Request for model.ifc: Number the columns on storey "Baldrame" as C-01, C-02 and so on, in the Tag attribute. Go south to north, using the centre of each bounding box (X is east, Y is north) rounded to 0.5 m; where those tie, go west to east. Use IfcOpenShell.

First a look at what the model holds.

```python
import ifcopenshell
import ifcopenshell.util.element
import ifcopenshell.util.placement

model = ifcopenshell.open("model.ifc")
print(model.schema)
storey = next(s for s in model.by_type("IfcBuildingStorey") if s.Name == "Baldrame")
columns = [e for e in ifcopenshell.util.element.get_decomposition(storey) if e.is_a("IfcColumn")]
for e in sorted(columns, key=lambda e: e.id()):
    origin = ifcopenshell.util.placement.get_local_placement(e.ObjectPlacement)[:3, 3]
    print(e.id(), e.Tag, e.Name, origin.round(2) + 0.0, sep=" | ")
```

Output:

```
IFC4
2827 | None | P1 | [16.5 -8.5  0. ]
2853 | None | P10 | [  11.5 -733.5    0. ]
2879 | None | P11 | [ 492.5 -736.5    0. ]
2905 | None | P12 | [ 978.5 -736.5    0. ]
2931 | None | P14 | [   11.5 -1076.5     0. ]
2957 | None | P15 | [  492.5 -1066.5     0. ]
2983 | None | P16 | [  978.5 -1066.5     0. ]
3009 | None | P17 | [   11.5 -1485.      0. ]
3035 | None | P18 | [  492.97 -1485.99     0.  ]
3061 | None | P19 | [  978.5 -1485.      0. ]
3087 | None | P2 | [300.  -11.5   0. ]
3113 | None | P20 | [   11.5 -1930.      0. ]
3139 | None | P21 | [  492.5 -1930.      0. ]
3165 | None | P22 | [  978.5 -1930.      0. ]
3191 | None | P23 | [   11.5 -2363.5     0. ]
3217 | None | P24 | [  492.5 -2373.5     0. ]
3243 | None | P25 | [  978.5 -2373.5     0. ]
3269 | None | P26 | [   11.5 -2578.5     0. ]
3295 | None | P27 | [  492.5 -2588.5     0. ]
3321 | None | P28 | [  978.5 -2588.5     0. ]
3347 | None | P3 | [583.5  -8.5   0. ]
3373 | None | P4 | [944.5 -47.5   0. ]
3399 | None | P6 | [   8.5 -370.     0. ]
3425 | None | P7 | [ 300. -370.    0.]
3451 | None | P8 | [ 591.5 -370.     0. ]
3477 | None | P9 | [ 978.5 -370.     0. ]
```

```python
import ifcopenshell
import ifcopenshell.geom
import ifcopenshell.util.element
import ifcopenshell.util.shape

model = ifcopenshell.open("model.ifc")
settings = ifcopenshell.geom.settings()
settings.set("use-world-coords", True)


def centre(element):
    shape = ifcopenshell.geom.create_shape(settings, element)
    return ifcopenshell.util.shape.get_bbox_centroid(shape.geometry)


storey = next(s for s in model.by_type("IfcBuildingStorey") if s.Name == "Baldrame")
columns = [e for e in ifcopenshell.util.element.get_decomposition(storey) if e.is_a("IfcColumn")]

# Insertion points can sit at a corner or the storey origin, so sort by the geometry (in metres).
centres = {e: centre(e) for e in columns}
columns.sort(key=lambda e: (round(centres[e][1] / 0.5), centres[e][0]))

for i, e in enumerate(columns, start=1):
    number = f"C-{i:02d}"
    e.Tag = number
    print(e.id(), number)

model.write("model_updated.ifc")
```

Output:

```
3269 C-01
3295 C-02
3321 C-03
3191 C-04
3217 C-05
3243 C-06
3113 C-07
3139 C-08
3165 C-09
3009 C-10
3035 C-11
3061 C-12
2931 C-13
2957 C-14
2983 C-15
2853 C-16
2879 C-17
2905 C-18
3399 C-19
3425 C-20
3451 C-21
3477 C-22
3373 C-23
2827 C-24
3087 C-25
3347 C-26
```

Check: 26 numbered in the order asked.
